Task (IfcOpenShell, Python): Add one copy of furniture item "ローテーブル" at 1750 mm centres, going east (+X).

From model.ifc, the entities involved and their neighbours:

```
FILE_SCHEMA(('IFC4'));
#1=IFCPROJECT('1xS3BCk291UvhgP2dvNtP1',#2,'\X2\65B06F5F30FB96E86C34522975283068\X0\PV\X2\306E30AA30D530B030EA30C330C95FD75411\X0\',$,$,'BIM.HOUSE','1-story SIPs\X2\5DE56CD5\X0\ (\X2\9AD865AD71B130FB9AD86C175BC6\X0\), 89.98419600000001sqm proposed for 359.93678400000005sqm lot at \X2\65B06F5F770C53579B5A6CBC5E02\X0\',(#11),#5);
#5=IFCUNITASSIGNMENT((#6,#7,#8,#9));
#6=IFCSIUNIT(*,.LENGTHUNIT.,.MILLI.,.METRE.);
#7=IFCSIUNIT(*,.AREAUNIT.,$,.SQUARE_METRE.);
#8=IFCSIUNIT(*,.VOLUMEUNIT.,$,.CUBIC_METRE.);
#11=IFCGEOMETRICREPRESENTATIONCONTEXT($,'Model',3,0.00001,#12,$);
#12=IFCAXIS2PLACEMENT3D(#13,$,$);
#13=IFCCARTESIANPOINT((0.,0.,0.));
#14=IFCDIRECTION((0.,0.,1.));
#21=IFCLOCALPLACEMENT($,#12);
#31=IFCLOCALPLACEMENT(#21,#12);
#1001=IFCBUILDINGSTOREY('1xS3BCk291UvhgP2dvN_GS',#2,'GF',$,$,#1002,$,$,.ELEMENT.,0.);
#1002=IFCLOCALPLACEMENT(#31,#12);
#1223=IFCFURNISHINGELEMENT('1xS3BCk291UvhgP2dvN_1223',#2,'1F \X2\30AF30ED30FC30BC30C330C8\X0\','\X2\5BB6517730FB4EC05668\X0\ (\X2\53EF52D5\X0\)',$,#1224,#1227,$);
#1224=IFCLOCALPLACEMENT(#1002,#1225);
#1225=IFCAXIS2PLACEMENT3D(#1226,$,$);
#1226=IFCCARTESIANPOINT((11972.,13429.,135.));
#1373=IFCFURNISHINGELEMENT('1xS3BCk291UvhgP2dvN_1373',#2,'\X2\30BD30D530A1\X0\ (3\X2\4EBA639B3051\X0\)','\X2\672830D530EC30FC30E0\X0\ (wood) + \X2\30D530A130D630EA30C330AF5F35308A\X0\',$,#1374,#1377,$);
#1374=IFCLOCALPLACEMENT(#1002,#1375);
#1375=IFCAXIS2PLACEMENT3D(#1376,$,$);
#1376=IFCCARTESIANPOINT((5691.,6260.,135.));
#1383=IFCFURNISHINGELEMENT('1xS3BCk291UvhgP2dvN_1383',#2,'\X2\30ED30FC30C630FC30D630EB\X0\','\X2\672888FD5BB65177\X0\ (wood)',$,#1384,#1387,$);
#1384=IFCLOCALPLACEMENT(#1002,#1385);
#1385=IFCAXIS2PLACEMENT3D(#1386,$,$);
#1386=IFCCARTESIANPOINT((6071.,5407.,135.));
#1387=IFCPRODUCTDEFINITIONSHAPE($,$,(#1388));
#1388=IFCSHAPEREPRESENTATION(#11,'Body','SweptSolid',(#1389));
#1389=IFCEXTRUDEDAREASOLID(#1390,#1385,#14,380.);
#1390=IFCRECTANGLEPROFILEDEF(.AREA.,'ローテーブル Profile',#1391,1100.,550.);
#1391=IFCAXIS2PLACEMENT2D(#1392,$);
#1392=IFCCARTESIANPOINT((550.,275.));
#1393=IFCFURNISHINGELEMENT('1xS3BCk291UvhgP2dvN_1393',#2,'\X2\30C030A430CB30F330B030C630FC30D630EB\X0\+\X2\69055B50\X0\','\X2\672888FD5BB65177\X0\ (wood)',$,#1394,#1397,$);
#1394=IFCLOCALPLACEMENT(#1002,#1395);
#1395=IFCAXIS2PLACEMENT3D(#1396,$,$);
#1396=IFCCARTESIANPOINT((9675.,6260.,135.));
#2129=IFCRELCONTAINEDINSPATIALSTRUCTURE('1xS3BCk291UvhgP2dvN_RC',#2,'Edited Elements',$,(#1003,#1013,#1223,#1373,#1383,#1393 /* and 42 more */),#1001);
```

```python
import numpy as np
import ifcopenshell
import ifcopenshell.api.geometry
import ifcopenshell.api.root
import ifcopenshell.util.element
import ifcopenshell.util.placement
import ifcopenshell.util.unit

model = ifcopenshell.open("model.ifc")
unit_scale = ifcopenshell.util.unit.calculate_unit_scale(model)


def reuse_history(source, copy):
    """copy_class also copies each property set's owner history, people and application; keep the originals."""
    for rel in copy.IsDefinedBy:
        if rel.is_a("IfcRelDefinesByProperties") and (history := rel.RelatingPropertyDefinition.OwnerHistory):
            rel.RelatingPropertyDefinition.OwnerHistory = source.OwnerHistory
            ifcopenshell.util.element.remove_deep2(model, history)


source = model.by_guid("1xS3BCk291UvhgP2dvN_1383")
base = ifcopenshell.util.placement.get_local_placement(source.ObjectPlacement)
step = np.array([1.0, 0.0, 0.0]) * 1.75 / unit_scale

for i in range(1, 2):
    copy = ifcopenshell.api.root.copy_class(model, product=source)
    copy.Representation = ifcopenshell.util.element.copy_deep(
        model, source.Representation, exclude=["IfcGeometricRepresentationContext", "IfcRepresentationMap"]
    )
    reuse_history(source, copy)
    matrix = base.copy()
    matrix[:3, 3] += i * step
    print("added at", matrix[:3, 3].round(3) + 0.0)
    ifcopenshell.api.geometry.edit_object_placement(model, product=copy, matrix=matrix, is_si=False)

model.write("model_v2.ifc")
```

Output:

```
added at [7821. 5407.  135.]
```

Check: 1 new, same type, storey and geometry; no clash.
